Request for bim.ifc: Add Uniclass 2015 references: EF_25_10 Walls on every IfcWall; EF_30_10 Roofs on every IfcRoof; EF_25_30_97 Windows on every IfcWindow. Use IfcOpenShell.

First a look at what the model holds.

```python
import ifcopenshell

model = ifcopenshell.open("bim.ifc")
print(model.schema)
print("classifications:", [c.Name for c in model.by_type("IfcClassification")])
for ifc_class in ("IfcDoor", "IfcRoof", "IfcStair", "IfcWall", "IfcWindow"):
    print(ifc_class, len(model.by_type(ifc_class)))
```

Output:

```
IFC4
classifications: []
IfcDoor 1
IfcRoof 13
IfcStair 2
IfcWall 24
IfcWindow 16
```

```python
import ifcopenshell
import ifcopenshell.api.classification

model = ifcopenshell.open("bim.ifc")

system = ifcopenshell.api.classification.add_classification(model, classification="Uniclass 2015")

codes = {
    "IfcWall": ("EF_25_10", "Walls"),
    "IfcRoof": ("EF_30_10", "Roofs"),
    "IfcWindow": ("EF_25_30_97", "Windows"),
}
for ifc_class, (code, name) in codes.items():
    products = model.by_type(ifc_class)
    ifcopenshell.api.classification.add_reference(
        model, products=products, classification=system, identification=code, name=name
    )
    print(code, len(products))

model.write("bim_edited.ifc")
```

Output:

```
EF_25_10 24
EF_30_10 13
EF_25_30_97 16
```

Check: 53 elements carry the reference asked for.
